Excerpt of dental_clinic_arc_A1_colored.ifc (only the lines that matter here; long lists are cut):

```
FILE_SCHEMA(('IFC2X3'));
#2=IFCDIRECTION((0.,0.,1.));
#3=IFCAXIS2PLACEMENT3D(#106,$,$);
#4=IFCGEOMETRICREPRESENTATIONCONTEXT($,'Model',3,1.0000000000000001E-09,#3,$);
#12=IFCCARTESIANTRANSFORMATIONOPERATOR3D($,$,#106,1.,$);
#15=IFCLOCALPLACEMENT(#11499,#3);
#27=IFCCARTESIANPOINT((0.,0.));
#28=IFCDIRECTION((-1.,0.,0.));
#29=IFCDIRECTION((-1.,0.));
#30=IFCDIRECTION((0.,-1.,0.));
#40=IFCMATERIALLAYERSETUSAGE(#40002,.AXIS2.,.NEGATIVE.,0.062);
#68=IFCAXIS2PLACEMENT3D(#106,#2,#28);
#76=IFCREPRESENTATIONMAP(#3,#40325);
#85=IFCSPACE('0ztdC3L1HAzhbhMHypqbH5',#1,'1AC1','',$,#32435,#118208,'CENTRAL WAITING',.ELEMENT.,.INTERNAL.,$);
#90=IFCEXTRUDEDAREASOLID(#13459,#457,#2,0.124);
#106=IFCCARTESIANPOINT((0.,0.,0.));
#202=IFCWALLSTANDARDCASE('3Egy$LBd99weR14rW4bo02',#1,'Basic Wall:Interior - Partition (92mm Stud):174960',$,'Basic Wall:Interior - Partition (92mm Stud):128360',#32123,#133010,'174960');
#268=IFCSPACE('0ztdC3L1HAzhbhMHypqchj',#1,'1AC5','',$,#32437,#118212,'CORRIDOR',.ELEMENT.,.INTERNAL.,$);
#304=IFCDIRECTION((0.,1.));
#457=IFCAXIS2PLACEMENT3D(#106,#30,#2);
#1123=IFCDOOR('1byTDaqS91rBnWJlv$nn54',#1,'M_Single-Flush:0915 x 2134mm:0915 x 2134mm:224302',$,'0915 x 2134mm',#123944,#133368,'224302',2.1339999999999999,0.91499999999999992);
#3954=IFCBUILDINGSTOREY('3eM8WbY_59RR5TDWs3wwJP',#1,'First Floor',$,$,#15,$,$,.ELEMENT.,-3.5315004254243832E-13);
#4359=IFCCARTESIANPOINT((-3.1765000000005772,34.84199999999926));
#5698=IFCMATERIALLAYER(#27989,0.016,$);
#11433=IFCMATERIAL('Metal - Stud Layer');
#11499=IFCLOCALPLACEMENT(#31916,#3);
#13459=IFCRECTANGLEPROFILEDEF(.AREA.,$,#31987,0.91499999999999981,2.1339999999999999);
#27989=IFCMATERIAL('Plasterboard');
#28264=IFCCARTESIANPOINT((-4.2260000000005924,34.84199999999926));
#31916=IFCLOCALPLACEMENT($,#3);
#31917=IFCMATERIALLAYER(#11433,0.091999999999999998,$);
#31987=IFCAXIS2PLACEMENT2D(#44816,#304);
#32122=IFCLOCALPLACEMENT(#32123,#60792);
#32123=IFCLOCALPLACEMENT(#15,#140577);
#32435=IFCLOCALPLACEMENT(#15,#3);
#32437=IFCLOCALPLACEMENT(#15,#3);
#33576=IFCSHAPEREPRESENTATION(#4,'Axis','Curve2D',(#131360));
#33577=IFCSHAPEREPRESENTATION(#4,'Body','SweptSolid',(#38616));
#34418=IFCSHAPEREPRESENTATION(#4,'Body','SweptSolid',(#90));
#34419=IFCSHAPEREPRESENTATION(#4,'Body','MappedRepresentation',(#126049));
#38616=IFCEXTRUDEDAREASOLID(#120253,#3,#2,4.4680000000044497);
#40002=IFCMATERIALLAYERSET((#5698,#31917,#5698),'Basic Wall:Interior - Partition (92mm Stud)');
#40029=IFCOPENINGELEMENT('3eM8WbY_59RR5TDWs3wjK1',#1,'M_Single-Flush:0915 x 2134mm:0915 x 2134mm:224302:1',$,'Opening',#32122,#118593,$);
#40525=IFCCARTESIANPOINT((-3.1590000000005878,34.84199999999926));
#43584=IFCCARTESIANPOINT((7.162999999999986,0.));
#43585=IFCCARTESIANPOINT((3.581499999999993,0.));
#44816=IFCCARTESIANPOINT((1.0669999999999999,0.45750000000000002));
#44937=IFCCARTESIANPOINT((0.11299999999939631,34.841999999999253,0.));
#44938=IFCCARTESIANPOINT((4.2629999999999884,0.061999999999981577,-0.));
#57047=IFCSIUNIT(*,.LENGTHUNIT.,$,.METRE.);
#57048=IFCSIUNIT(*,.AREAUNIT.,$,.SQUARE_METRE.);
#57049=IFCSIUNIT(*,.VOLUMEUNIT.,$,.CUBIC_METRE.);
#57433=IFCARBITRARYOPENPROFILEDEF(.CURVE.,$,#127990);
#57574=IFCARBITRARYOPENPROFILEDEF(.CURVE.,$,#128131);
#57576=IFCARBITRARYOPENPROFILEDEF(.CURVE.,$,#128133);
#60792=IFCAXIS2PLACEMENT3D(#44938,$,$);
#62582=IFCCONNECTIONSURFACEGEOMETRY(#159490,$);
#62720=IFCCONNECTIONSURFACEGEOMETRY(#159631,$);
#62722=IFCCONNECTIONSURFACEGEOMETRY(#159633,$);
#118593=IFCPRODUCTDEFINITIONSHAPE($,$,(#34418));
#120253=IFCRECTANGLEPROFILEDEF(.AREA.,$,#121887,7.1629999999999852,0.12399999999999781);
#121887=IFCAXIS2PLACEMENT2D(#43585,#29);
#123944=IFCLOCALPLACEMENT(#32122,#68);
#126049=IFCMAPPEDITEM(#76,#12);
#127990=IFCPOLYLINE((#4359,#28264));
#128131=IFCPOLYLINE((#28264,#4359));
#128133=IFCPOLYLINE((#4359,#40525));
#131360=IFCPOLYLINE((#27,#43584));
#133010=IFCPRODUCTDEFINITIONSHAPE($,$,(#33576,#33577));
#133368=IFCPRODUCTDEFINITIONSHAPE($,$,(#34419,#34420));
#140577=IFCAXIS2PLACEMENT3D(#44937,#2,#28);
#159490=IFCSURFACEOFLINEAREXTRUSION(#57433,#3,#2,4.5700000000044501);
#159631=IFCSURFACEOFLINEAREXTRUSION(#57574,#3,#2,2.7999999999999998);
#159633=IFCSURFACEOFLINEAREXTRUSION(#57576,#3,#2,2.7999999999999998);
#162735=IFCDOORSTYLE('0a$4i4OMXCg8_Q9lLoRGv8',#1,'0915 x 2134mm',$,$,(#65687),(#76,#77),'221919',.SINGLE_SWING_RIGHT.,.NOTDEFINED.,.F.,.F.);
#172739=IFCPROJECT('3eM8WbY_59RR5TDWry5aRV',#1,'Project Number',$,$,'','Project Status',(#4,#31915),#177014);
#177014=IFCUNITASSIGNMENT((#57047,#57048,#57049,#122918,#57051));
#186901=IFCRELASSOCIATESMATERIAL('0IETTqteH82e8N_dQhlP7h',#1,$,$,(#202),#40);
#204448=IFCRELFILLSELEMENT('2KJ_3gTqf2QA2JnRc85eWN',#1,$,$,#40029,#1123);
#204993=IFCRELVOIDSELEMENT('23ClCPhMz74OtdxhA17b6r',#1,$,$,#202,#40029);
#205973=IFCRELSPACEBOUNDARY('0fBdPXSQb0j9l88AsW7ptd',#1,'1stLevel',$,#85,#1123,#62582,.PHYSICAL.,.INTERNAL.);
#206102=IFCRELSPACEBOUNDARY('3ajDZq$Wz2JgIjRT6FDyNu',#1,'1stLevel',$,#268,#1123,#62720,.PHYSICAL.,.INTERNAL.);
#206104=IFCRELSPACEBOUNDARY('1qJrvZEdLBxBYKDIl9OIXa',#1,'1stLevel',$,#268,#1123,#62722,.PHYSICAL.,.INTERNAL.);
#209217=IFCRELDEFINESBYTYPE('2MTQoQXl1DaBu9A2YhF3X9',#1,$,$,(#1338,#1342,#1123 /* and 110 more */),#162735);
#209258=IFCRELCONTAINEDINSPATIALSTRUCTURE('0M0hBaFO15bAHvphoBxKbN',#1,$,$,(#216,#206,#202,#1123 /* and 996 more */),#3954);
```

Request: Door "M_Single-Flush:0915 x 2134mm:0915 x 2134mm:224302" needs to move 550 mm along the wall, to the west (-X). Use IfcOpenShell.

```python
import numpy as np
import ifcopenshell
import ifcopenshell.api.geometry
import ifcopenshell.util.placement
import ifcopenshell.util.unit

model = ifcopenshell.open("dental_clinic_arc_A1_colored.ifc")
unit_scale = ifcopenshell.util.unit.calculate_unit_scale(model)

door = model.by_guid("1byTDaqS91rBnWJlv$nn54")
opening = door.FillsVoids[0].RelatingOpeningElement
wall = opening.VoidsElements[0].RelatingBuildingElement

wall_matrix = ifcopenshell.util.placement.get_local_placement(wall.ObjectPlacement)
shift = wall_matrix[:3, 0] * 0.55 / unit_scale
before = ifcopenshell.util.placement.get_local_placement(door.ObjectPlacement)[:3, 3].copy()

# The door is placed relative to its opening, so it follows when the opening moves.
matrix = ifcopenshell.util.placement.get_local_placement(opening.ObjectPlacement)
matrix[:3, 3] += shift
ifcopenshell.api.geometry.edit_object_placement(
    model, product=opening, matrix=matrix, is_si=False, should_transform_children=True
)

# Space boundary surfaces are stored in each space's coordinates; move them too.
for rel in door.ProvidesBoundaries:
    if not rel.ConnectionGeometry:
        continue
    surface = rel.ConnectionGeometry.SurfaceOnRelatingElement
    space_matrix = ifcopenshell.util.placement.get_local_placement(rel.RelatingSpace.ObjectPlacement)
    point = np.array(surface.Position.Location.Coordinates) + space_matrix[:3, :3].T @ shift
    surface.Position = model.createIfcAxis2Placement3D(
        model.createIfcCartesianPoint(point.tolist()), surface.Position.Axis, surface.Position.RefDirection
    )

after = ifcopenshell.util.placement.get_local_placement(door.ObjectPlacement)[:3, 3]
print("door moved by", (after - before).round(3) + 0.0)

model.write("dental_clinic_arc_A1_colored_updated.ifc")
```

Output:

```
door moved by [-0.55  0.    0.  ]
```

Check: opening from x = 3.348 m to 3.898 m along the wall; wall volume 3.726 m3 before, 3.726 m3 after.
